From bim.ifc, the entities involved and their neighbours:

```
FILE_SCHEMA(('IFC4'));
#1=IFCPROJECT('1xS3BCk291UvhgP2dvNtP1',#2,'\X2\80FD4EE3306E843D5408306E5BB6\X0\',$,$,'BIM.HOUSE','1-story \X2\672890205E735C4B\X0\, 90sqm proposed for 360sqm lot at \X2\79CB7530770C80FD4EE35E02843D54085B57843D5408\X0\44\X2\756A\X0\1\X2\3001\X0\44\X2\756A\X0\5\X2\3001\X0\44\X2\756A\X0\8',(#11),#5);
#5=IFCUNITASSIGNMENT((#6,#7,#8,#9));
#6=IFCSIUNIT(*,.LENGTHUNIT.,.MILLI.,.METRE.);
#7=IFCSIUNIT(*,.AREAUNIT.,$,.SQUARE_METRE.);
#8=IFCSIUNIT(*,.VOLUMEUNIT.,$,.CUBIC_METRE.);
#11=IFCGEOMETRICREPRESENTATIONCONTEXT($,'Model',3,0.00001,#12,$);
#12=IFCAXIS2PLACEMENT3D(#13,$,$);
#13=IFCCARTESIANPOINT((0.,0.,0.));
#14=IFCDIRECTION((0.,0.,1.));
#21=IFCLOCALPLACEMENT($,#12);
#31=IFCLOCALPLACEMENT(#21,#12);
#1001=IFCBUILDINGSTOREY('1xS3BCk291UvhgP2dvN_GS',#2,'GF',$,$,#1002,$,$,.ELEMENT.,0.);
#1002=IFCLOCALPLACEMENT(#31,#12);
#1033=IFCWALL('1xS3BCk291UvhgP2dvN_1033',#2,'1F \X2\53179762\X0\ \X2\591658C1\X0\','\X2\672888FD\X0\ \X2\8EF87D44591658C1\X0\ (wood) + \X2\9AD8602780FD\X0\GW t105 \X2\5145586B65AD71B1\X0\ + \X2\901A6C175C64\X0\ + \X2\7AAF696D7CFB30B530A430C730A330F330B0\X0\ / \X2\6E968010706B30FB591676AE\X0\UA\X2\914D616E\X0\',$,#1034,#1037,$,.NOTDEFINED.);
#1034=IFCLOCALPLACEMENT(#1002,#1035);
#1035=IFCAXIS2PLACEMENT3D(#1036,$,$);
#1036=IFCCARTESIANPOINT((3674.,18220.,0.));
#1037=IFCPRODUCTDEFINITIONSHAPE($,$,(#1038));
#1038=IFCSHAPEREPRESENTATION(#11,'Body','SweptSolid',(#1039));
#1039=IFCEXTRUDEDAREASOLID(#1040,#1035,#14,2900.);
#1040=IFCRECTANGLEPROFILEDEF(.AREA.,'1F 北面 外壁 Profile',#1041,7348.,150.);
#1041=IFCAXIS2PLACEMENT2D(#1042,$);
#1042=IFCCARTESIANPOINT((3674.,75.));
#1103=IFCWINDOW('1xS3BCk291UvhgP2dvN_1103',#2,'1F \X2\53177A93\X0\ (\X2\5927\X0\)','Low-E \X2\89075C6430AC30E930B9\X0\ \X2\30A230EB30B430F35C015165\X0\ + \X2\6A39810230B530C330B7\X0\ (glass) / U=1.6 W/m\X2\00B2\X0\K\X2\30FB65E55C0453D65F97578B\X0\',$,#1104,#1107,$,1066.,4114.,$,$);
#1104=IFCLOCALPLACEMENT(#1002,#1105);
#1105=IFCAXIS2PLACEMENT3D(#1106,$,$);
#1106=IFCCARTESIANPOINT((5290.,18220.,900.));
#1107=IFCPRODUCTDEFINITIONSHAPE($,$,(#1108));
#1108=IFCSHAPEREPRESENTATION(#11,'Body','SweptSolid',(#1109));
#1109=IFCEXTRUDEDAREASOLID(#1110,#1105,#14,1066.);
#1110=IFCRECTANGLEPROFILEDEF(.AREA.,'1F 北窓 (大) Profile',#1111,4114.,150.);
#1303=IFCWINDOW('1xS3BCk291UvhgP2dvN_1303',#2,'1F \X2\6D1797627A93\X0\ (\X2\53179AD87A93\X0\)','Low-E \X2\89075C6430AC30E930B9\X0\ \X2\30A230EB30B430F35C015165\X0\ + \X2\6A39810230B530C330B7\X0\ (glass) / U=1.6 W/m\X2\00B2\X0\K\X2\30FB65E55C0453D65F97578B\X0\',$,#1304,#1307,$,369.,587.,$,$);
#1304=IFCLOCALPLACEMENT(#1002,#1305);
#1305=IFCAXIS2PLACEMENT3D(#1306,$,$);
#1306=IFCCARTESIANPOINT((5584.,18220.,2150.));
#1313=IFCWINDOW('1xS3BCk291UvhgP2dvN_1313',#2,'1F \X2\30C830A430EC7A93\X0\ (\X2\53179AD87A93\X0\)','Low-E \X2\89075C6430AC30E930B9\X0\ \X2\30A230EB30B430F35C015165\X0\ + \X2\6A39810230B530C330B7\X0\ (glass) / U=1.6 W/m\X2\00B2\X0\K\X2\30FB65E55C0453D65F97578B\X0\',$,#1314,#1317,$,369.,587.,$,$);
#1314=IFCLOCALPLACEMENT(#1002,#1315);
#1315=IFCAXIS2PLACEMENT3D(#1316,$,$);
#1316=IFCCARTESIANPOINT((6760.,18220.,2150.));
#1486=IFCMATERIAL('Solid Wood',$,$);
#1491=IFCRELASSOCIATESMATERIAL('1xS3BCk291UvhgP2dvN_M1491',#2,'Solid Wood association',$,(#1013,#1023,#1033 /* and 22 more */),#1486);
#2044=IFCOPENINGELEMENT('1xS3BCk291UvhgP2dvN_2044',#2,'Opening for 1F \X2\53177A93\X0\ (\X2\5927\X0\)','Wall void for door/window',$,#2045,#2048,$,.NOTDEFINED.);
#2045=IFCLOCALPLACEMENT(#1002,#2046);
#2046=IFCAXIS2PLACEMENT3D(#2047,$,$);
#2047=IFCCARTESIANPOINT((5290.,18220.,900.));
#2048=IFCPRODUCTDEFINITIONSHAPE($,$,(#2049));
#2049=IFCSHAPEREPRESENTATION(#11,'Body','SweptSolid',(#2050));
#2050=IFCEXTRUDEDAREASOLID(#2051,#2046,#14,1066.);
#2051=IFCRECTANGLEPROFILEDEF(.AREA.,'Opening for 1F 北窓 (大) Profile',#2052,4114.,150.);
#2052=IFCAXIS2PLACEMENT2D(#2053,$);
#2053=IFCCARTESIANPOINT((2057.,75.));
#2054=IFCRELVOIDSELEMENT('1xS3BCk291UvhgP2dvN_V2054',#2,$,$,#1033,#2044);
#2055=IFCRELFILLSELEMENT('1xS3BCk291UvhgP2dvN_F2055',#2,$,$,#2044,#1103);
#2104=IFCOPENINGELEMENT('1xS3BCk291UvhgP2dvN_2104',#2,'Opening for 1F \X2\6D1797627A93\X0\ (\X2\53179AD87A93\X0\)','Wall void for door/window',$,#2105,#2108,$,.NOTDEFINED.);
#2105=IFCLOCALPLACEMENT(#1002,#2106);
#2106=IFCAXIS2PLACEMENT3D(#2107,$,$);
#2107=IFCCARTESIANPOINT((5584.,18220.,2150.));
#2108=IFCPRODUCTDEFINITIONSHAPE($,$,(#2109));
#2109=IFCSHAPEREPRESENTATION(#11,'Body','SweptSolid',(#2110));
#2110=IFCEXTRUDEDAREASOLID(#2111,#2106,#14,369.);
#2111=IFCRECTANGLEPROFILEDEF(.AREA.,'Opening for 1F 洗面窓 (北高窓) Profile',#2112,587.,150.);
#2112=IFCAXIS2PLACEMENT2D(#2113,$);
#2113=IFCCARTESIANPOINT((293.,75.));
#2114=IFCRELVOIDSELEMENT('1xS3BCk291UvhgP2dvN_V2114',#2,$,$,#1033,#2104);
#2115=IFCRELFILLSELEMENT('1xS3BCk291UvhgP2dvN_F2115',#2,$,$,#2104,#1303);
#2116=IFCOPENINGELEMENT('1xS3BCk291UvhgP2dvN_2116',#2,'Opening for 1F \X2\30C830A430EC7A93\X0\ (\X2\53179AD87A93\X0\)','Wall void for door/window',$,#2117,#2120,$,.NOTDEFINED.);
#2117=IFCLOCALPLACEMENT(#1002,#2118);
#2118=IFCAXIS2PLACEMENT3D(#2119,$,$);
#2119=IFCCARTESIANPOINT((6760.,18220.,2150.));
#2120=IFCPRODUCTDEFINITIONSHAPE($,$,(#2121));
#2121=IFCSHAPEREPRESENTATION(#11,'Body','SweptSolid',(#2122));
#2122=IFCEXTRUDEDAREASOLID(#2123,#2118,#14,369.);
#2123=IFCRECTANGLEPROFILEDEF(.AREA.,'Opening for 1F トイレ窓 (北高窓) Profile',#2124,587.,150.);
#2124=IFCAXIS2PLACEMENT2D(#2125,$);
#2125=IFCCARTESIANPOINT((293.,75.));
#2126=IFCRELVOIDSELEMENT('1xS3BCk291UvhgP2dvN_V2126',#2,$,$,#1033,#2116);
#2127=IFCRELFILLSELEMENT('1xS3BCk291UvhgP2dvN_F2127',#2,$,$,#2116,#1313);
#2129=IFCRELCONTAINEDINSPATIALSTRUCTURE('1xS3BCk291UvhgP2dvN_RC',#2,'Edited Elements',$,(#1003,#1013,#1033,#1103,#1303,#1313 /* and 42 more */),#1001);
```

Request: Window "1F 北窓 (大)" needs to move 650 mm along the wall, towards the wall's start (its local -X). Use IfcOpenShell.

```python
import ifcopenshell
import ifcopenshell.api.geometry
import ifcopenshell.util.placement

model = ifcopenshell.open("bim.ifc")

window = model.by_guid("1xS3BCk291UvhgP2dvN_1103")
opening = window.FillsVoids[0].RelatingOpeningElement
wall = opening.VoidsElements[0].RelatingBuildingElement

wall_matrix = ifcopenshell.util.placement.get_local_placement(wall.ObjectPlacement)
shift = wall_matrix[:3, 0] * -650.0
before = ifcopenshell.util.placement.get_local_placement(window.ObjectPlacement)[:3, 3].copy()

# The window is not placed relative to its opening, so move both.
for product in (opening, window):
    matrix = ifcopenshell.util.placement.get_local_placement(product.ObjectPlacement)
    matrix[:3, 3] += shift
    ifcopenshell.api.geometry.edit_object_placement(model, product=product, matrix=matrix, is_si=False)

after = ifcopenshell.util.placement.get_local_placement(window.ObjectPlacement)[:3, 3]
print("window moved by", (after - before).round(3) + 0.0)

model.write("bim_updated.ifc")
```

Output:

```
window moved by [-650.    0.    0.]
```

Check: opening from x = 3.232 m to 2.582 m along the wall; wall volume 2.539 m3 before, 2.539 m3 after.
